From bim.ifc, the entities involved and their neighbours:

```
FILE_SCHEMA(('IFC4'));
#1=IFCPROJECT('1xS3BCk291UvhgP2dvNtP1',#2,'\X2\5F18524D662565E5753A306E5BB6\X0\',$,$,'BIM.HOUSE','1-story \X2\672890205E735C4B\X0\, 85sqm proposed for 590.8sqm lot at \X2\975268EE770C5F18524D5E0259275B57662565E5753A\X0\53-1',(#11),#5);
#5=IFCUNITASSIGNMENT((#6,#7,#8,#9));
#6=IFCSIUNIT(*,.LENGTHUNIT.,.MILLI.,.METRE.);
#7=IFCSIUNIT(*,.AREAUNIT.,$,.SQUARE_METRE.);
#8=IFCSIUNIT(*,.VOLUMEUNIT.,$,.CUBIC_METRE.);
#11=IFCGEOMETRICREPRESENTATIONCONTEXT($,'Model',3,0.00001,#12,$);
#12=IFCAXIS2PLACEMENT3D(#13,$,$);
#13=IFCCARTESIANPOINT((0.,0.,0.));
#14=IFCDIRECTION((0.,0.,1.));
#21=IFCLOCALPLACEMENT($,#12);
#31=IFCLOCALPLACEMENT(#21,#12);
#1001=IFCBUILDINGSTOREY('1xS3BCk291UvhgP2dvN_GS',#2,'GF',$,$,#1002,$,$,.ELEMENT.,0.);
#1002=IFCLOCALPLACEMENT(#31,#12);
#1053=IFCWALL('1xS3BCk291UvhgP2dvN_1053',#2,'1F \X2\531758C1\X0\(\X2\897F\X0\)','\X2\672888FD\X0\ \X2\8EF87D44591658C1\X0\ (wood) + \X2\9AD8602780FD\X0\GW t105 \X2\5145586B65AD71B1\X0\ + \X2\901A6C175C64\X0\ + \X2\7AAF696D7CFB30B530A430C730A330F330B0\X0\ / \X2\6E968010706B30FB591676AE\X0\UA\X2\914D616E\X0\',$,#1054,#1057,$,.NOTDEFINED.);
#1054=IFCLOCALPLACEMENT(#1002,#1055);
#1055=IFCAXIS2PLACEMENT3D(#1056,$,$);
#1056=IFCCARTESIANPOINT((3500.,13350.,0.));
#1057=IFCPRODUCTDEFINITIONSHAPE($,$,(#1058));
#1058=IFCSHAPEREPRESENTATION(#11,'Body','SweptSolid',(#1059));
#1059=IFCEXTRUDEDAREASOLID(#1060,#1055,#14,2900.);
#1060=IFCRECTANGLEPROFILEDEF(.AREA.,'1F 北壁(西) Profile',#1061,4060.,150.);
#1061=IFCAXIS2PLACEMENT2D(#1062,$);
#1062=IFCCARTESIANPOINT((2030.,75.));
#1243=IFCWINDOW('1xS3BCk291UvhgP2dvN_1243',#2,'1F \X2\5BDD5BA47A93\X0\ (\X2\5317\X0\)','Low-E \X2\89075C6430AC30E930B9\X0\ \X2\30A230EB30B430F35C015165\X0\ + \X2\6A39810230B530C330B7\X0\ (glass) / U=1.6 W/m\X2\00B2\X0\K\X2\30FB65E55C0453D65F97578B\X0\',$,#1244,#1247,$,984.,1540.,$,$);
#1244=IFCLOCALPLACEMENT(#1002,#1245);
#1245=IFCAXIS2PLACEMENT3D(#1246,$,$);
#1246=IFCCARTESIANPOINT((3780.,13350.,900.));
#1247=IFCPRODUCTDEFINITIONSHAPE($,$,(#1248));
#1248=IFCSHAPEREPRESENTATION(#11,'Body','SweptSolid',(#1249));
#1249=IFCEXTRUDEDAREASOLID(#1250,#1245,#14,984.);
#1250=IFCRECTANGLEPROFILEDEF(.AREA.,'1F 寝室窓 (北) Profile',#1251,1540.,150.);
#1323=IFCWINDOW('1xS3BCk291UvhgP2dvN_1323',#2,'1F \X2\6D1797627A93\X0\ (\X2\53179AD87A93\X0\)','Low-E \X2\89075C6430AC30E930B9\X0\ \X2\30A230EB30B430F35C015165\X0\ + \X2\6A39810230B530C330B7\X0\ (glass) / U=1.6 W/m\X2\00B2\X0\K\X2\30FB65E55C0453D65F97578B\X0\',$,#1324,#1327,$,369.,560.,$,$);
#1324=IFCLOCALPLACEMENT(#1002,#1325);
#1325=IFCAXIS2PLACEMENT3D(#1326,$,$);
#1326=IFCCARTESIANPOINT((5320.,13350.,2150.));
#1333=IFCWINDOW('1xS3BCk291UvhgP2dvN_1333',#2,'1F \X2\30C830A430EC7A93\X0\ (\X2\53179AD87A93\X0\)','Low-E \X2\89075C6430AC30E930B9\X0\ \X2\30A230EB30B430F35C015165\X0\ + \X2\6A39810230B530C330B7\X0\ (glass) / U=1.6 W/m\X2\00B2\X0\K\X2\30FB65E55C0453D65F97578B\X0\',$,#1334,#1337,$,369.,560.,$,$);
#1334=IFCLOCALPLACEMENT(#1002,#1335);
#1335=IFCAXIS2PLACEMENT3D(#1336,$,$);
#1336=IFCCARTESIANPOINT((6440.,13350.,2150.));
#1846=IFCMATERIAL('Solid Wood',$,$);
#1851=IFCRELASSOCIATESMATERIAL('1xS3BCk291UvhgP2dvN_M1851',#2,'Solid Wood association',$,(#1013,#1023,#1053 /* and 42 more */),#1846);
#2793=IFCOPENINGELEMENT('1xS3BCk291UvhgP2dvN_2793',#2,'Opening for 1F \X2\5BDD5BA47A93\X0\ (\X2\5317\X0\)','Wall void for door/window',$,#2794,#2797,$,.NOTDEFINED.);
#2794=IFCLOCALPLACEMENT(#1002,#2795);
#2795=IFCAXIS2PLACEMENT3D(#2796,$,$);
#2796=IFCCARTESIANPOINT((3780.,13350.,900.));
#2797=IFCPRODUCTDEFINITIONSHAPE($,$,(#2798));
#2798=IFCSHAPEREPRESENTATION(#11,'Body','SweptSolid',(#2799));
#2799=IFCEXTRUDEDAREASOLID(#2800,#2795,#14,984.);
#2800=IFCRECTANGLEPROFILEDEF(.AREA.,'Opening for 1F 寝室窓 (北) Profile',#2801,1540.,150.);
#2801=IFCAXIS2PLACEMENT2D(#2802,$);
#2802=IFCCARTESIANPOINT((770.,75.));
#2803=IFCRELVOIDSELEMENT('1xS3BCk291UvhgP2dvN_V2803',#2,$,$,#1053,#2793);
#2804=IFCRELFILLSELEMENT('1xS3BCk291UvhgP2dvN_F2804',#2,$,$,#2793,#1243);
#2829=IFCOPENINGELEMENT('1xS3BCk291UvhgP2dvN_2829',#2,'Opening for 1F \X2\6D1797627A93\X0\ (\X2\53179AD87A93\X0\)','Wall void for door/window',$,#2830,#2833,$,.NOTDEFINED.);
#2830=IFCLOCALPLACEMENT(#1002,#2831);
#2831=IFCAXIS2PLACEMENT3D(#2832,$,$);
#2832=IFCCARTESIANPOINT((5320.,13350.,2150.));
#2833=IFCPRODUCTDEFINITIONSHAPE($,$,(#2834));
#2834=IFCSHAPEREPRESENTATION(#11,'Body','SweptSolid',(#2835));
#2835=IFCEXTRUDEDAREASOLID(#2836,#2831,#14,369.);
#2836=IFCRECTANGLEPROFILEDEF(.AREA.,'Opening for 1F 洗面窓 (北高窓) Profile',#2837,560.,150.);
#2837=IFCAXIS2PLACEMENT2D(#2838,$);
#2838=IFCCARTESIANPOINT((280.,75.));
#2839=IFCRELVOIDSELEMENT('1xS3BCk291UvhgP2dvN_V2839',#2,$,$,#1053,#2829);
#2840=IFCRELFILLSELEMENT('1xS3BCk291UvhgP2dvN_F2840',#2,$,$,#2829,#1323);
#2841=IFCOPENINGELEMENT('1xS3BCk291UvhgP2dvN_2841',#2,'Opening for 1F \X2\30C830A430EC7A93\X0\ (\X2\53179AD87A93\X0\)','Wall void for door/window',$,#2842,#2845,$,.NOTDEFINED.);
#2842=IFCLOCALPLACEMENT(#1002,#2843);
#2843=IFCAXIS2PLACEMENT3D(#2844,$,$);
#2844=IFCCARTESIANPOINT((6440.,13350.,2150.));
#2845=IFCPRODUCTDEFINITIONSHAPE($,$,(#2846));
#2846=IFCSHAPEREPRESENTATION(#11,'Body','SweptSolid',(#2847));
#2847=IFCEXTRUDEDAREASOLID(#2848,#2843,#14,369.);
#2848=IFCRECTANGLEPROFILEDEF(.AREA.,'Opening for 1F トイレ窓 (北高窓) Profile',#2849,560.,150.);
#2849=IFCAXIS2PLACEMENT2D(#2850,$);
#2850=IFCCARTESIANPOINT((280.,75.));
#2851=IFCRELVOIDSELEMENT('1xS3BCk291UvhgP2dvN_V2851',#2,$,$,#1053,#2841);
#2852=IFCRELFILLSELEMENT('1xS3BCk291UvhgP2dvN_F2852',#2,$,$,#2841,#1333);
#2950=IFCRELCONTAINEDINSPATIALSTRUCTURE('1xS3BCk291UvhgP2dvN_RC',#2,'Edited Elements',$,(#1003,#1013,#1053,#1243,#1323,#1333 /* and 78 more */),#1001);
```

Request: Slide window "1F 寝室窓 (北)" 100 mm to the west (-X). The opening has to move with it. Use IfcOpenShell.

```python
import ifcopenshell
import ifcopenshell.api.geometry
import ifcopenshell.util.placement

model = ifcopenshell.open("bim.ifc")

window = model.by_guid("1xS3BCk291UvhgP2dvN_1243")
opening = window.FillsVoids[0].RelatingOpeningElement
wall = opening.VoidsElements[0].RelatingBuildingElement

wall_matrix = ifcopenshell.util.placement.get_local_placement(wall.ObjectPlacement)
shift = wall_matrix[:3, 0] * -100.0
before = ifcopenshell.util.placement.get_local_placement(window.ObjectPlacement)[:3, 3].copy()

# The window is not placed relative to its opening, so move both.
for product in (opening, window):
    matrix = ifcopenshell.util.placement.get_local_placement(product.ObjectPlacement)
    matrix[:3, 3] += shift
    ifcopenshell.api.geometry.edit_object_placement(model, product=product, matrix=matrix, is_si=False)

after = ifcopenshell.util.placement.get_local_placement(window.ObjectPlacement)[:3, 3]
print("window moved by", (after - before).round(3) + 0.0)

model.write("bim_rev.ifc")
```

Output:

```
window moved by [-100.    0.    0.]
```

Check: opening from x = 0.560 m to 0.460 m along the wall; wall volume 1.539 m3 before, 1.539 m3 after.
